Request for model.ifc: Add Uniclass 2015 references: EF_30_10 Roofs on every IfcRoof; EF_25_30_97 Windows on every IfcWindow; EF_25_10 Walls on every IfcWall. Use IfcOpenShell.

First a look at what the model holds.

```python
import ifcopenshell

model = ifcopenshell.open("model.ifc")
print(model.schema)
print("classifications:", [c.Name for c in model.by_type("IfcClassification")])
for ifc_class in ("IfcDoor", "IfcRoof", "IfcStair", "IfcWall", "IfcWindow"):
    print(ifc_class, len(model.by_type(ifc_class)))
```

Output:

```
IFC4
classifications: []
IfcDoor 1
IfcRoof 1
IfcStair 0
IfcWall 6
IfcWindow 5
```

```python
import ifcopenshell
import ifcopenshell.api.classification

model = ifcopenshell.open("model.ifc")

system = ifcopenshell.api.classification.add_classification(model, classification="Uniclass 2015")

codes = {
    "IfcRoof": ("EF_30_10", "Roofs"),
    "IfcWindow": ("EF_25_30_97", "Windows"),
    "IfcWall": ("EF_25_10", "Walls"),
}
for ifc_class, (code, name) in codes.items():
    products = model.by_type(ifc_class)
    ifcopenshell.api.classification.add_reference(
        model, products=products, classification=system, identification=code, name=name
    )
    print(code, len(products))

model.write("model_v2.ifc")
```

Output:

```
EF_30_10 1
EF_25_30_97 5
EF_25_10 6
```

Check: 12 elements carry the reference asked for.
